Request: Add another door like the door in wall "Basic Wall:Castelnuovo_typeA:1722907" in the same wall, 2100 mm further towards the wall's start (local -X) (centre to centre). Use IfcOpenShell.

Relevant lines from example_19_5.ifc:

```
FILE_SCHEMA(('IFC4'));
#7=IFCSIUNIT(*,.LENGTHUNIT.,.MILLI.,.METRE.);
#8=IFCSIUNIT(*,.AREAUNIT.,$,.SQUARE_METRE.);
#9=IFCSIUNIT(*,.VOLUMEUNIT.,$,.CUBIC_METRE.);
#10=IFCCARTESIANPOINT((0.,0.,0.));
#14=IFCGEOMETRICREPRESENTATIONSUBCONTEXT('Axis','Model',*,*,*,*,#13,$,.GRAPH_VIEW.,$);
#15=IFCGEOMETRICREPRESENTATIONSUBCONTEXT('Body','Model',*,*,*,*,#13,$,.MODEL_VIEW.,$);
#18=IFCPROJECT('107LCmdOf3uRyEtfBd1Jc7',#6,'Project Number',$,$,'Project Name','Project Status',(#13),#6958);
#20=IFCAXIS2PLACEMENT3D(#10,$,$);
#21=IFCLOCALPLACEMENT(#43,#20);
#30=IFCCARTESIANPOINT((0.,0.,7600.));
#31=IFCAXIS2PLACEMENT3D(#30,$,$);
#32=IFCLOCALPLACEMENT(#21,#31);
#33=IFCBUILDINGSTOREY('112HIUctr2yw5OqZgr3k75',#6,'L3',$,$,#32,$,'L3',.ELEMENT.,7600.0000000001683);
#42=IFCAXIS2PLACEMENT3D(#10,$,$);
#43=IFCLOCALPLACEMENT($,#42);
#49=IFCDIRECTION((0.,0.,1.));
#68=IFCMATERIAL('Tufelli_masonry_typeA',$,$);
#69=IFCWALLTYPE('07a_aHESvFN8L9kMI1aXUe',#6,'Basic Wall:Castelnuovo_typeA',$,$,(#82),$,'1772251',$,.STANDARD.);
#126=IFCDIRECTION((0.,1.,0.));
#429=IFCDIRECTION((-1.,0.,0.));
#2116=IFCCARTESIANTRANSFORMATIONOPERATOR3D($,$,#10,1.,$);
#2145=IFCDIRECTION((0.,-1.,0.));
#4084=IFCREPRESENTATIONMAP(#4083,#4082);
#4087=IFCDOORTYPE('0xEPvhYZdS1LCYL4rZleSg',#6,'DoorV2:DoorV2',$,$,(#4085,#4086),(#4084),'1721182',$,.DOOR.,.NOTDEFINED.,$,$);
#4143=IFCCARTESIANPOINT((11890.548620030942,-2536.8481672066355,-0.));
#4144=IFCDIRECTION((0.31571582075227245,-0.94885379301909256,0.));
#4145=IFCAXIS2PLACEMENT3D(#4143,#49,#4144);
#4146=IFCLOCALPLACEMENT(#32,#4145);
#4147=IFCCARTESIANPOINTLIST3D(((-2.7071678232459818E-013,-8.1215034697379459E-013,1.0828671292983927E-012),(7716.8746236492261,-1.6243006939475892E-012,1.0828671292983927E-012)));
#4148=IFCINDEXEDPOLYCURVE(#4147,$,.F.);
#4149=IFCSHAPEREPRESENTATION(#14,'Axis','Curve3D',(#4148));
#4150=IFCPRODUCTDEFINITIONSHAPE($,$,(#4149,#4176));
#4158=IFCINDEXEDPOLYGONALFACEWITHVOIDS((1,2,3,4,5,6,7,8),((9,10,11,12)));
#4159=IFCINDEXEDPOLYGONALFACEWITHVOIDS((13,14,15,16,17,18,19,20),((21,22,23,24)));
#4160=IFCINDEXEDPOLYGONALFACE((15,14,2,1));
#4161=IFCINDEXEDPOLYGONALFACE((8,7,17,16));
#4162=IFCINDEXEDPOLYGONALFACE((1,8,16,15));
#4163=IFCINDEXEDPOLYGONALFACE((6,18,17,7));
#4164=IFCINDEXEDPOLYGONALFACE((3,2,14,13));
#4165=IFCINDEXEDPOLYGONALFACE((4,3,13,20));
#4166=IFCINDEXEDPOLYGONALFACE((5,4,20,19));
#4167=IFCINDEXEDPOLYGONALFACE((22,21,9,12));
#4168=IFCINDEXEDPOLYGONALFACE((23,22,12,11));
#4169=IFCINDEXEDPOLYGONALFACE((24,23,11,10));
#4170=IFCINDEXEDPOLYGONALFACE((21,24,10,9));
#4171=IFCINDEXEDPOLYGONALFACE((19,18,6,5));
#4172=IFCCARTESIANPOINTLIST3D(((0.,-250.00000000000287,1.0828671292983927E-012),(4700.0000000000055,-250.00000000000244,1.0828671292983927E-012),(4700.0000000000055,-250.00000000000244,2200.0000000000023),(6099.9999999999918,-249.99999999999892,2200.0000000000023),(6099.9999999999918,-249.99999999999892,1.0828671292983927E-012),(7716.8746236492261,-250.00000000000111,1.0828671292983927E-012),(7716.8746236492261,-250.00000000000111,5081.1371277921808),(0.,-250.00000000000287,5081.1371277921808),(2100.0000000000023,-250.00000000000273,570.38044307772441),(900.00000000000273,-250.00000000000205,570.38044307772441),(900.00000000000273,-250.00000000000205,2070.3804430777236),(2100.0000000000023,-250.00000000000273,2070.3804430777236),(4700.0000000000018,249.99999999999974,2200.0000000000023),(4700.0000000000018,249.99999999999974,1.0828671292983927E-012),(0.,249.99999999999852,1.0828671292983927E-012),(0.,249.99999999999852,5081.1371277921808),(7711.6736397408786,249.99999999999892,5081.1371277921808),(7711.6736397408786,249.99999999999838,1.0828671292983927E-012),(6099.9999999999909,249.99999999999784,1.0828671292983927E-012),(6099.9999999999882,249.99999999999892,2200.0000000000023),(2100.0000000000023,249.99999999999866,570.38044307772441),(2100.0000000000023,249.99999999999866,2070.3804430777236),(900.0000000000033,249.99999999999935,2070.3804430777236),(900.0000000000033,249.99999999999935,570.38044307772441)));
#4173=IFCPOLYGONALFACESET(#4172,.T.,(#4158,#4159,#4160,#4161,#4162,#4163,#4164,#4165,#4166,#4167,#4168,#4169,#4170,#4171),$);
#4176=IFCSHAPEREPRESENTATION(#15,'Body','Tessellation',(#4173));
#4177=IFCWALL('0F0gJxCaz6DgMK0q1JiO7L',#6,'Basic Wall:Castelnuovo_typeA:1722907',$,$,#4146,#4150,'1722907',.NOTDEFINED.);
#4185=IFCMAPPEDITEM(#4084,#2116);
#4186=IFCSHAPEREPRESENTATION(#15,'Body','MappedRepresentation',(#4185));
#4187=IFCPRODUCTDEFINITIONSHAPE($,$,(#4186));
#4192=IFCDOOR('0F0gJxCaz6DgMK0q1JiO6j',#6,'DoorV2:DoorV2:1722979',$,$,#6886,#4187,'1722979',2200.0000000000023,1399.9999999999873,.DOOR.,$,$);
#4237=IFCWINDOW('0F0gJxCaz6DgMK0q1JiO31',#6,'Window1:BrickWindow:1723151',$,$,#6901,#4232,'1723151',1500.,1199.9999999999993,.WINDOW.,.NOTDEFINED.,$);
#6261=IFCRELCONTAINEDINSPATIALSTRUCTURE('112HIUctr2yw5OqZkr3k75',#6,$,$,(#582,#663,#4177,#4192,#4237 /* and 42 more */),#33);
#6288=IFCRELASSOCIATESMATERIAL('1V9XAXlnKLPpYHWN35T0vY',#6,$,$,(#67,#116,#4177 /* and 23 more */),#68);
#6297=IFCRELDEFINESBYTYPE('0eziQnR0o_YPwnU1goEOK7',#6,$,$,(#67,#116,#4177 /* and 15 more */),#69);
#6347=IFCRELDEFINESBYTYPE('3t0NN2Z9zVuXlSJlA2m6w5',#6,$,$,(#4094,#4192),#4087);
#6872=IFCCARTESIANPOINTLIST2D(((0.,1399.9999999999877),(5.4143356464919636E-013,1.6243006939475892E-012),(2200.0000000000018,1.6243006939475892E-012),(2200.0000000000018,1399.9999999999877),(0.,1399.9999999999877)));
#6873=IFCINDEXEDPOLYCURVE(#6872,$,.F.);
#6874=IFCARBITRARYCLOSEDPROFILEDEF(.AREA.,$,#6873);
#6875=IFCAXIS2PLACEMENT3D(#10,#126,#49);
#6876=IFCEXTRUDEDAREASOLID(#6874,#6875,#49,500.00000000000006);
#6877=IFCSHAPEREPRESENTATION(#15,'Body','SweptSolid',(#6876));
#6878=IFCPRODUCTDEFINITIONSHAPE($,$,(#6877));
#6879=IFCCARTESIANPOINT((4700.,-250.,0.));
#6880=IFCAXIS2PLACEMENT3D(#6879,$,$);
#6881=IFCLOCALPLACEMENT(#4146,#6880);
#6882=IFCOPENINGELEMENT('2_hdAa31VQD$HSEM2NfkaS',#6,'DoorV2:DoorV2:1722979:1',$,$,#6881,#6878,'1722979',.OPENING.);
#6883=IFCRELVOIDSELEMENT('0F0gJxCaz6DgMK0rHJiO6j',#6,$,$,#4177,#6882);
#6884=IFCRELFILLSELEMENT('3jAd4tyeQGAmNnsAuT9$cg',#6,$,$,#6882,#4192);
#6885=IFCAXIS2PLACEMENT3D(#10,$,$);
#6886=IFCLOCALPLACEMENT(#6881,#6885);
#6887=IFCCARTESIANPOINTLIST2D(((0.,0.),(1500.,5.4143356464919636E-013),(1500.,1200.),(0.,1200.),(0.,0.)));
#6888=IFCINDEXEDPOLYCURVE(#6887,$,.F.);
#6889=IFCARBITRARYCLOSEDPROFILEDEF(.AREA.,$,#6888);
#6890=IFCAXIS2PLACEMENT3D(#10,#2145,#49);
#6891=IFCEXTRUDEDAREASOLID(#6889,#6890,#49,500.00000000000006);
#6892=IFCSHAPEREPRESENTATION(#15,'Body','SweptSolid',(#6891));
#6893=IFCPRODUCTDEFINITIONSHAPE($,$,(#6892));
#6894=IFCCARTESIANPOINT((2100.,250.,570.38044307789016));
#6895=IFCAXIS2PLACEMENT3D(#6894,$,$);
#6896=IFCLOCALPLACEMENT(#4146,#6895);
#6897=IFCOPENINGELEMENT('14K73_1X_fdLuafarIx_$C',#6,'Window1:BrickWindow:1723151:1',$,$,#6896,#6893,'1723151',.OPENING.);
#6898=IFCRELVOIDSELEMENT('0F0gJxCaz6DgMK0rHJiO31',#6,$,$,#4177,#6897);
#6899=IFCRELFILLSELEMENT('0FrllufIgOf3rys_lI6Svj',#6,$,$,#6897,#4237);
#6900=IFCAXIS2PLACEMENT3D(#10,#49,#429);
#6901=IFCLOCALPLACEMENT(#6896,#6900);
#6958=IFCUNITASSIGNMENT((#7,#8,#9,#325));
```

```python
import ifcopenshell
import ifcopenshell.api.feature
import ifcopenshell.api.geometry
import ifcopenshell.api.root
import ifcopenshell.geom
import ifcopenshell.util.element
import ifcopenshell.util.placement
import ifcopenshell.util.shape

model = ifcopenshell.open("example_19_5.ifc")
settings = ifcopenshell.geom.settings()


def volume(element):
    """Net volume in cubic metres, openings subtracted."""
    shape = ifcopenshell.geom.create_shape(settings, element)
    return ifcopenshell.util.shape.get_volume(shape.geometry)


def reuse_history(source, copy):
    """copy_class also copies each property set's owner history, people and application; keep the originals."""
    for rel in copy.IsDefinedBy:
        if rel.is_a("IfcRelDefinesByProperties") and (history := rel.RelatingPropertyDefinition.OwnerHistory):
            rel.RelatingPropertyDefinition.OwnerHistory = source.OwnerHistory
            ifcopenshell.util.element.remove_deep2(model, history)


door = model.by_id(4192)
opening = door.FillsVoids[0].RelatingOpeningElement
wall = opening.VoidsElements[0].RelatingBuildingElement
before = volume(wall)
shift = ifcopenshell.util.placement.get_local_placement(wall.ObjectPlacement)[:3, 0] * -2100.0

# copy_class copies the void relationship, type, container and properties, but no geometry.
new_opening = ifcopenshell.api.root.copy_class(model, product=opening)
new_opening.Representation = ifcopenshell.util.element.copy_deep(
    model, opening.Representation, exclude=["IfcGeometricRepresentationContext", "IfcRepresentationMap"]
)
new_opening.Name = "DoorV2:DoorV2"
new_opening.Tag = None
new_door = ifcopenshell.api.root.copy_class(model, product=door)
new_door.Representation = ifcopenshell.util.element.copy_deep(
    model, door.Representation, exclude=["IfcGeometricRepresentationContext", "IfcRepresentationMap"]
)
new_door.Name = "DoorV2:DoorV2"
new_door.Tag = None
reuse_history(door, new_door)
ifcopenshell.api.feature.add_filling(model, opening=new_opening, element=new_door)

for old, new in ((opening, new_opening), (door, new_door)):
    matrix = ifcopenshell.util.placement.get_local_placement(old.ObjectPlacement)
    matrix[:3, 3] += shift
    ifcopenshell.api.geometry.edit_object_placement(model, product=new, matrix=matrix, is_si=False)

after = volume(wall)

print(f"wall volume {before:.3f} -> {after:.3f} m3")

model.write("example_19_5_updated.ifc")
```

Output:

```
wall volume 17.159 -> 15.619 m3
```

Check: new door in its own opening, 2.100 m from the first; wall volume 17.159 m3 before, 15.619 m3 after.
